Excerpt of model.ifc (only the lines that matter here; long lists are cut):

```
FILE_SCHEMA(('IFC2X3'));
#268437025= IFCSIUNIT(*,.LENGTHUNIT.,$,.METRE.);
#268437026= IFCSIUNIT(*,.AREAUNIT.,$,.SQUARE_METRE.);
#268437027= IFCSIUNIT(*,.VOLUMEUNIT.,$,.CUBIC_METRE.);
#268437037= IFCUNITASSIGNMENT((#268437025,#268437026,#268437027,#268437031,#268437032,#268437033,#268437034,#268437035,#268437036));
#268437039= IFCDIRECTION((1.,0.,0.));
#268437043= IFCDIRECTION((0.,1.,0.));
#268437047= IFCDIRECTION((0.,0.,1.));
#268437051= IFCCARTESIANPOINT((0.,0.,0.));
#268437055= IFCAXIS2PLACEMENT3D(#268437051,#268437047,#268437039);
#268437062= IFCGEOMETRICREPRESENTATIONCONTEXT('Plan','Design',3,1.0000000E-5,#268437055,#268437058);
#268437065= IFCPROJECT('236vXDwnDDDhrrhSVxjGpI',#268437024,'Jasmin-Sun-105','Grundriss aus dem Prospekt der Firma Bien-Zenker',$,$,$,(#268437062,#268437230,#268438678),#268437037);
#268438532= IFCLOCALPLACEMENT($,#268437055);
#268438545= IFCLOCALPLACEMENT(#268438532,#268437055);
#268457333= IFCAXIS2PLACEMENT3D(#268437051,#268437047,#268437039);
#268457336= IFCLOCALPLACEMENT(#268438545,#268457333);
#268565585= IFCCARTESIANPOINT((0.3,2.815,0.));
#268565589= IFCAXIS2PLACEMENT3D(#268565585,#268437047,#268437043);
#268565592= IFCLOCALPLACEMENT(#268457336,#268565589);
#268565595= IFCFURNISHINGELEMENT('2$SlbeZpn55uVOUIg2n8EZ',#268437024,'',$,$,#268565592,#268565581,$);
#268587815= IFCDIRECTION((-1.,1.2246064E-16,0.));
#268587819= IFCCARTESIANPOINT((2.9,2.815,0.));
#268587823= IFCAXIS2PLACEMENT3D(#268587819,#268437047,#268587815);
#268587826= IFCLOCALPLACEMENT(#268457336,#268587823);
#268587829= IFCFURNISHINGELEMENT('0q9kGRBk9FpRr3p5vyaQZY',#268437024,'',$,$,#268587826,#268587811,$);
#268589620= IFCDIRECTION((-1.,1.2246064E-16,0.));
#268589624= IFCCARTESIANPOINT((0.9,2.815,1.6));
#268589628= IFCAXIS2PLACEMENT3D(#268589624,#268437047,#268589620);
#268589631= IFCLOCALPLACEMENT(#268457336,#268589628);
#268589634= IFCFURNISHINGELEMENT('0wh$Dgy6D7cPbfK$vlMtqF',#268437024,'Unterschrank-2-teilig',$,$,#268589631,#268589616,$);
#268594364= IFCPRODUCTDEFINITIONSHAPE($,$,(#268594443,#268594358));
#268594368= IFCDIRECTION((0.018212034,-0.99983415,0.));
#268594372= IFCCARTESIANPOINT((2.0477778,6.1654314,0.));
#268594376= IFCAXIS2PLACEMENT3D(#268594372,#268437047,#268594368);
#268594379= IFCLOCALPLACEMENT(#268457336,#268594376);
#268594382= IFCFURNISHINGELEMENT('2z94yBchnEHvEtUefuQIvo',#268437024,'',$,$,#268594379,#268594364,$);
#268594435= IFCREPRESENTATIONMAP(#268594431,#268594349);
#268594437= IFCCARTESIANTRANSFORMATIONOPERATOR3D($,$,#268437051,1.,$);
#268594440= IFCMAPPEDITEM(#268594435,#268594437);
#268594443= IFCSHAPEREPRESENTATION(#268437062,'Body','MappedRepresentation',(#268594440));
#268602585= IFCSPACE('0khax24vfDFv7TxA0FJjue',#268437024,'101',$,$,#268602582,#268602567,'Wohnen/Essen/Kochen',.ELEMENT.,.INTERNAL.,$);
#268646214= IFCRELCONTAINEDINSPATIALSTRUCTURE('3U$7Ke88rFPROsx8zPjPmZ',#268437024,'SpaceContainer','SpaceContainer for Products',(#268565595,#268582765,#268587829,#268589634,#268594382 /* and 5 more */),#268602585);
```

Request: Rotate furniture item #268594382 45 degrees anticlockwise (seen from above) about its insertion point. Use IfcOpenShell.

```python
import ifcopenshell
import ifcopenshell.api.geometry
import ifcopenshell.util.placement

model = ifcopenshell.open("model.ifc")

item = model.by_guid("2z94yBchnEHvEtUefuQIvo")
matrix = ifcopenshell.util.placement.get_local_placement(item.ObjectPlacement)
matrix = matrix @ ifcopenshell.util.placement.rotation(45, "Z")
ifcopenshell.api.geometry.edit_object_placement(model, product=item, matrix=matrix, is_si=False)

print(ifcopenshell.util.placement.get_local_placement(item.ObjectPlacement).round(3) + 0.0)

model.write("model_edited.ifc")
```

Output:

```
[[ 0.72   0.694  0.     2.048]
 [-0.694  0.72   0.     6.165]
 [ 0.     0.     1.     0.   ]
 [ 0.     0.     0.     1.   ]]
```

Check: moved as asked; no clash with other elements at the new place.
